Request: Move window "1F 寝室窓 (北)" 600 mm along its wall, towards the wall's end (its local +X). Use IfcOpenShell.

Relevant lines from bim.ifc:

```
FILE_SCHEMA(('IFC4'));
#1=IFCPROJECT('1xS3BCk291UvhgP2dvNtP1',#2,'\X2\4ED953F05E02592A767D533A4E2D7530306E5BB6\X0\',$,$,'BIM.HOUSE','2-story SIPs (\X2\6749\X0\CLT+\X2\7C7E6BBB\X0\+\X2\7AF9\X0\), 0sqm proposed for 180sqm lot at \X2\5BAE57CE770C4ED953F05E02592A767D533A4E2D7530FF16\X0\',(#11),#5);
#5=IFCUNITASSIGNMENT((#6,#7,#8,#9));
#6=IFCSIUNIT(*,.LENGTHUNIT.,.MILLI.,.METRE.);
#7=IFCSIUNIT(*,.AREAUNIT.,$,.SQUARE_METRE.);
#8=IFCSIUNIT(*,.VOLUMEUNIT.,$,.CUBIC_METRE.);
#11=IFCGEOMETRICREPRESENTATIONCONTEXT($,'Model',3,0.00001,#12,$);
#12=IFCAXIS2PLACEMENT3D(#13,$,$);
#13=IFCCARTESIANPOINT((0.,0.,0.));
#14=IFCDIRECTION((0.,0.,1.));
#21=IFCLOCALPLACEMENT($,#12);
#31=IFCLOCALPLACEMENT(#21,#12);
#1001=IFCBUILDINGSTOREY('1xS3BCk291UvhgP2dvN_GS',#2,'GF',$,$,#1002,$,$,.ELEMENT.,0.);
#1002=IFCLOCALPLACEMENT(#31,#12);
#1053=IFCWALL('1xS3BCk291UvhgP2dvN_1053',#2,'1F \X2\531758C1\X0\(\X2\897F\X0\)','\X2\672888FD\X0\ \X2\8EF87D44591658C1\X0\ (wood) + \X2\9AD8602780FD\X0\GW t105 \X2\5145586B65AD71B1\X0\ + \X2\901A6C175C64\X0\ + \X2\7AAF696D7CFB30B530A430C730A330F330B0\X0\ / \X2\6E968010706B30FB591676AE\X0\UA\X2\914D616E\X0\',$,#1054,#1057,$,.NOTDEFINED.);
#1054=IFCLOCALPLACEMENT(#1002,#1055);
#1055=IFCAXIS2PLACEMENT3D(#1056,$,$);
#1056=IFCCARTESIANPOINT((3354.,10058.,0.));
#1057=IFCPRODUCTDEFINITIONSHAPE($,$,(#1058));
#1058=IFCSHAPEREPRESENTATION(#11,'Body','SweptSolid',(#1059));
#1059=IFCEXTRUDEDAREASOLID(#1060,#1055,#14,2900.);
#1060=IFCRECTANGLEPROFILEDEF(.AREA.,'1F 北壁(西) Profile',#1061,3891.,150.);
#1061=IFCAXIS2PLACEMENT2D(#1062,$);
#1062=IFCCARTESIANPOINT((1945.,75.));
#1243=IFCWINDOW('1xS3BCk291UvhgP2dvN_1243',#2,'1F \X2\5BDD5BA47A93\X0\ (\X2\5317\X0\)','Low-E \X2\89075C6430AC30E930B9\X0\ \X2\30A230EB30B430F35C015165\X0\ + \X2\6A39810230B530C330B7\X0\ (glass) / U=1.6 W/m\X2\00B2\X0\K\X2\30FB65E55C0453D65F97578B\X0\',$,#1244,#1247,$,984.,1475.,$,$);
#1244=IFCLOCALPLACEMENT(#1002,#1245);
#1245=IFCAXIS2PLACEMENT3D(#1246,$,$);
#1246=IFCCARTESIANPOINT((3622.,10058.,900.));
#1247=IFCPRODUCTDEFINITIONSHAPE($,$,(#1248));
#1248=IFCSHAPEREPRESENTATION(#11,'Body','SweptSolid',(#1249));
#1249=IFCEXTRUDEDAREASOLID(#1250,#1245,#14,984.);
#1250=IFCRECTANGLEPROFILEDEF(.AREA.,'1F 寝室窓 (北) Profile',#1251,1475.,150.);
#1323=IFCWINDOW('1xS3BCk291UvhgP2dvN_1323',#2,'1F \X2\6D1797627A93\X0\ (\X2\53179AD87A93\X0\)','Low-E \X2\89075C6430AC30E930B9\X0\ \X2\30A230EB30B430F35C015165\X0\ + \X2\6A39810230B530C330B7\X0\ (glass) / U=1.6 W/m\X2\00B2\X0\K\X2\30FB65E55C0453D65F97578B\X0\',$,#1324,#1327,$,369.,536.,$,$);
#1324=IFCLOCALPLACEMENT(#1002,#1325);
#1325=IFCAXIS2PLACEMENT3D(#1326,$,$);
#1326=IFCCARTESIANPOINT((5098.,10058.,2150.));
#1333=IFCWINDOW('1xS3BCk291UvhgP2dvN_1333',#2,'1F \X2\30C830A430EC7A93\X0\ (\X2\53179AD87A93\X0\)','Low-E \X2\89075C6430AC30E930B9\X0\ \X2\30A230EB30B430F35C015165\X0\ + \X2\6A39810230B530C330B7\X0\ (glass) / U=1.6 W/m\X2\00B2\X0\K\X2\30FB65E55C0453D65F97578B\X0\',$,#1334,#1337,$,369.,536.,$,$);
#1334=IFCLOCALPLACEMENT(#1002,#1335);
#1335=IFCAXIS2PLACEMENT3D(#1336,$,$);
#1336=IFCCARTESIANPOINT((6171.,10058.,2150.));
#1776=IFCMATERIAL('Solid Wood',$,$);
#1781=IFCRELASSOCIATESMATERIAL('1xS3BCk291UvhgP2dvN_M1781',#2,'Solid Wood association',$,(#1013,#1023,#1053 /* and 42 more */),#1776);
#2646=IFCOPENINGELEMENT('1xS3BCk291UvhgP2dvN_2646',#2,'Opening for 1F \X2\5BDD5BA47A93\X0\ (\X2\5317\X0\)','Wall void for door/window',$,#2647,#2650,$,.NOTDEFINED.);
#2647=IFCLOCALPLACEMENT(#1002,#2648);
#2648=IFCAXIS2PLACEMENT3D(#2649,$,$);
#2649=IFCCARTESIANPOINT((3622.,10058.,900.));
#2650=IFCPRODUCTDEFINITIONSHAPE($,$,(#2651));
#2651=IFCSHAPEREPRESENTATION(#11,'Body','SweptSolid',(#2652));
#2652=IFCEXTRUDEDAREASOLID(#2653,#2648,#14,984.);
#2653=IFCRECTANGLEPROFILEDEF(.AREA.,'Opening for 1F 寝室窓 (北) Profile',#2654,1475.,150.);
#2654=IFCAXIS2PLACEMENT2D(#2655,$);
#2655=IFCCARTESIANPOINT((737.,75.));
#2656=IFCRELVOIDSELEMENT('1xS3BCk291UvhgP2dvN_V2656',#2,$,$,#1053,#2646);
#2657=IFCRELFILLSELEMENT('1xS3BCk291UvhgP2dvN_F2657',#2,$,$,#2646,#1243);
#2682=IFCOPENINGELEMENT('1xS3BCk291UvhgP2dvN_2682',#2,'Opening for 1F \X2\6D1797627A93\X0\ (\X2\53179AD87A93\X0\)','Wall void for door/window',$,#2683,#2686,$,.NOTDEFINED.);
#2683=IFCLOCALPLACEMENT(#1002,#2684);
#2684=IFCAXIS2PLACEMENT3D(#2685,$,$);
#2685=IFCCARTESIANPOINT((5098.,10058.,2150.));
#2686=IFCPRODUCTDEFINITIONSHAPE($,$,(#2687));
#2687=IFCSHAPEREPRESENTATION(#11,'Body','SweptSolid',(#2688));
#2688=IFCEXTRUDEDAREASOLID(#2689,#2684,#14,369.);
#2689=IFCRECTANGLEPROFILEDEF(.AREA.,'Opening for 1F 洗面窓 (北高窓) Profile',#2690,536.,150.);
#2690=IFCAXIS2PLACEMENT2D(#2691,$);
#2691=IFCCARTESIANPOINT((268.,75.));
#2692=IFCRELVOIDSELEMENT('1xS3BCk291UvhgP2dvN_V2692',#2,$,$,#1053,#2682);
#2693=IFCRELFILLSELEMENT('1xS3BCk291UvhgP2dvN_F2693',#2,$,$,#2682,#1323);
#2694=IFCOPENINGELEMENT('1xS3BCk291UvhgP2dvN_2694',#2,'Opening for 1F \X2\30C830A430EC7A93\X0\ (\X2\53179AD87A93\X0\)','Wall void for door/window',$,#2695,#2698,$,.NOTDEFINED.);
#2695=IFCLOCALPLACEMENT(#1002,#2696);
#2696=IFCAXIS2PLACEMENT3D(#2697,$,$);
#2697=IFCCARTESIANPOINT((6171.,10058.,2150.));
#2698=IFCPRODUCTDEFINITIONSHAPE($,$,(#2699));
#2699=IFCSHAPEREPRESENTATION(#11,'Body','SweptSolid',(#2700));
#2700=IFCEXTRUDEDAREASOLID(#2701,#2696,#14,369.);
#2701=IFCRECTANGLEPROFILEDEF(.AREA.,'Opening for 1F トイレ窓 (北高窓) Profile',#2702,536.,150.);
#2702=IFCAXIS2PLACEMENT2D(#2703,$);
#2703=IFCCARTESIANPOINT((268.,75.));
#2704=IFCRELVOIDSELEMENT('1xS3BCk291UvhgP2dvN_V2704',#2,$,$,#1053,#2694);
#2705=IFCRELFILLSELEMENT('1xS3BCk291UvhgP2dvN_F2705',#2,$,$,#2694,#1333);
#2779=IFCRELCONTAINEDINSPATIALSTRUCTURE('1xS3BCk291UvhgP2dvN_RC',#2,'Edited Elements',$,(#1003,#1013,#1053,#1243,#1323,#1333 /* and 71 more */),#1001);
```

```python
import ifcopenshell
import ifcopenshell.api.geometry
import ifcopenshell.util.placement
import ifcopenshell.util.unit

model = ifcopenshell.open("bim.ifc")
unit_scale = ifcopenshell.util.unit.calculate_unit_scale(model)

window = model.by_guid("1xS3BCk291UvhgP2dvN_1243")
opening = window.FillsVoids[0].RelatingOpeningElement
wall = opening.VoidsElements[0].RelatingBuildingElement

wall_matrix = ifcopenshell.util.placement.get_local_placement(wall.ObjectPlacement)
shift = wall_matrix[:3, 0] * 0.6 / unit_scale
before = ifcopenshell.util.placement.get_local_placement(window.ObjectPlacement)[:3, 3].copy()

# The window is not placed relative to its opening, so move both.
for product in (opening, window):
    matrix = ifcopenshell.util.placement.get_local_placement(product.ObjectPlacement)
    matrix[:3, 3] += shift
    ifcopenshell.api.geometry.edit_object_placement(model, product=product, matrix=matrix, is_si=False)

after = ifcopenshell.util.placement.get_local_placement(window.ObjectPlacement)[:3, 3]
print("window moved by", (after - before).round(3) + 0.0)

model.write("bim_v2.ifc")
```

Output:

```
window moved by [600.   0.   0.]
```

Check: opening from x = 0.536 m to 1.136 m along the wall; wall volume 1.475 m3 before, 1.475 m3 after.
